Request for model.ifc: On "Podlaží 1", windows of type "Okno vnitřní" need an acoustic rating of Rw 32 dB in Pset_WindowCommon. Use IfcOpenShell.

First a look at what the model holds.

```python
import ifcopenshell
import ifcopenshell.util.element

model = ifcopenshell.open("model.ifc")
print(model.schema)
storey = next(s for s in model.by_type("IfcBuildingStorey") if s.Name == "Podlaží 1")
windows = [e for e in ifcopenshell.util.element.get_decomposition(storey) if e.is_a("IfcWindow")]
seen = {}
for e in windows:
    element_type = ifcopenshell.util.element.get_type(e)
    key = (element_type.Name if element_type != e and element_type else None, ifcopenshell.util.element.get_pset(e, "Pset_WindowCommon", "AcousticRating"))
    seen[key] = seen.get(key, 0) + 1
for (name, value), count in sorted(seen.items(), key=str):
    print(count, "x", name, "|", value)
```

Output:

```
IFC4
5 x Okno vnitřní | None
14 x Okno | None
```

```python
import ifcopenshell
import ifcopenshell.api.pset
import ifcopenshell.util.element

model = ifcopenshell.open("model.ifc")

storey = next(s for s in model.by_type("IfcBuildingStorey") if s.Name == "Podlaží 1")
windows = [e for e in ifcopenshell.util.element.get_decomposition(storey) if e.is_a("IfcWindow")]

count = 0
for e in windows:
    element_type = ifcopenshell.util.element.get_type(e)
    if element_type in (None, e) or element_type.Name != "Okno vnitřní":
        continue
    # add_pset returns the element's existing set when there is one.
    pset = ifcopenshell.api.pset.add_pset(model, product=e, name="Pset_WindowCommon")
    ifcopenshell.api.pset.edit_pset(model, pset=pset, properties={"AcousticRating": "Rw 32 dB"})
    count += 1

print(count, "windows updated")

model.write("model_rev.ifc")
```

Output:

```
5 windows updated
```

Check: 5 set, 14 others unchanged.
